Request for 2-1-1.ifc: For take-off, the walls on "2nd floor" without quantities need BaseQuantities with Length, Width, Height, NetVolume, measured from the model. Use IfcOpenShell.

First a look at what the model holds.

```python
import ifcopenshell
import ifcopenshell.util.element
import ifcopenshell.util.unit

model = ifcopenshell.open("2-1-1.ifc")
print(model.schema)
for unit_type in ("LENGTHUNIT", "AREAUNIT", "VOLUMEUNIT"):
    print(unit_type, ifcopenshell.util.unit.calculate_unit_scale(model, unit_type))
storey = next(s for s in model.by_type("IfcBuildingStorey") if s.Name == "2nd floor")
walls = [e for e in ifcopenshell.util.element.get_decomposition(storey) if e.is_a("IfcWall")]
for e in sorted(walls, key=lambda e: e.id()):
    print(e.id(), e.is_a(), e.Name, list(ifcopenshell.util.element.get_psets(e, qtos_only=True)), sep=" | ")
```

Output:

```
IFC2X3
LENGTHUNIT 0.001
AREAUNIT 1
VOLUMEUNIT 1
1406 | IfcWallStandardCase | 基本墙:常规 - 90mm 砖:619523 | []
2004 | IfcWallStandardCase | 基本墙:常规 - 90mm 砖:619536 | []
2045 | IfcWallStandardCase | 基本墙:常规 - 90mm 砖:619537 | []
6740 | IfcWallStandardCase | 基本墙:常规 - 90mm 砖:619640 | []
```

```python
import ifcopenshell
import ifcopenshell.api.pset
import ifcopenshell.geom
import ifcopenshell.util.element
import ifcopenshell.util.shape
import ifcopenshell.util.unit

model = ifcopenshell.open("2-1-1.ifc")
unit_scale = ifcopenshell.util.unit.calculate_unit_scale(model)
volume_scale = ifcopenshell.util.unit.calculate_unit_scale(model, "VOLUMEUNIT")
settings = ifcopenshell.geom.settings()

storey = next(s for s in model.by_type("IfcBuildingStorey") if s.Name == "2nd floor")
walls = [e for e in ifcopenshell.util.element.get_decomposition(storey) if e.is_a("IfcWall")]

for e in sorted(walls, key=lambda e: e.id()):
    if ifcopenshell.util.element.get_psets(e, qtos_only=True, should_inherit=False):
        continue
    # Geometry comes back in metres, in the element's own axes.
    shape = ifcopenshell.geom.create_shape(settings, e)
    values = {
        "Length": ifcopenshell.util.shape.get_x(shape.geometry) / unit_scale,
        "Width": ifcopenshell.util.shape.get_y(shape.geometry) / unit_scale,
        "Height": ifcopenshell.util.shape.get_z(shape.geometry) / unit_scale,
        "NetVolume": ifcopenshell.util.shape.get_volume(shape.geometry) / volume_scale,
    }
    qto = ifcopenshell.api.pset.add_qto(model, product=e, name="BaseQuantities")
    ifcopenshell.api.pset.edit_qto(model, qto=qto, properties=values)
    print(e.id(), {k: round(v, 3) for k, v in values.items()})

model.write("2-1-1_updated.ifc")
```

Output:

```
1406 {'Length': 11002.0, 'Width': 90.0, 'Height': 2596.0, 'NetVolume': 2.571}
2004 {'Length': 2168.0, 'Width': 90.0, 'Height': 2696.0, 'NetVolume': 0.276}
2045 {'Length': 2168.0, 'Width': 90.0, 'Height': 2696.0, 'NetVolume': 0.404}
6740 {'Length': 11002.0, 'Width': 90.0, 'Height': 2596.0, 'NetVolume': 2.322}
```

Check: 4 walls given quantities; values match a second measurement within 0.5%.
